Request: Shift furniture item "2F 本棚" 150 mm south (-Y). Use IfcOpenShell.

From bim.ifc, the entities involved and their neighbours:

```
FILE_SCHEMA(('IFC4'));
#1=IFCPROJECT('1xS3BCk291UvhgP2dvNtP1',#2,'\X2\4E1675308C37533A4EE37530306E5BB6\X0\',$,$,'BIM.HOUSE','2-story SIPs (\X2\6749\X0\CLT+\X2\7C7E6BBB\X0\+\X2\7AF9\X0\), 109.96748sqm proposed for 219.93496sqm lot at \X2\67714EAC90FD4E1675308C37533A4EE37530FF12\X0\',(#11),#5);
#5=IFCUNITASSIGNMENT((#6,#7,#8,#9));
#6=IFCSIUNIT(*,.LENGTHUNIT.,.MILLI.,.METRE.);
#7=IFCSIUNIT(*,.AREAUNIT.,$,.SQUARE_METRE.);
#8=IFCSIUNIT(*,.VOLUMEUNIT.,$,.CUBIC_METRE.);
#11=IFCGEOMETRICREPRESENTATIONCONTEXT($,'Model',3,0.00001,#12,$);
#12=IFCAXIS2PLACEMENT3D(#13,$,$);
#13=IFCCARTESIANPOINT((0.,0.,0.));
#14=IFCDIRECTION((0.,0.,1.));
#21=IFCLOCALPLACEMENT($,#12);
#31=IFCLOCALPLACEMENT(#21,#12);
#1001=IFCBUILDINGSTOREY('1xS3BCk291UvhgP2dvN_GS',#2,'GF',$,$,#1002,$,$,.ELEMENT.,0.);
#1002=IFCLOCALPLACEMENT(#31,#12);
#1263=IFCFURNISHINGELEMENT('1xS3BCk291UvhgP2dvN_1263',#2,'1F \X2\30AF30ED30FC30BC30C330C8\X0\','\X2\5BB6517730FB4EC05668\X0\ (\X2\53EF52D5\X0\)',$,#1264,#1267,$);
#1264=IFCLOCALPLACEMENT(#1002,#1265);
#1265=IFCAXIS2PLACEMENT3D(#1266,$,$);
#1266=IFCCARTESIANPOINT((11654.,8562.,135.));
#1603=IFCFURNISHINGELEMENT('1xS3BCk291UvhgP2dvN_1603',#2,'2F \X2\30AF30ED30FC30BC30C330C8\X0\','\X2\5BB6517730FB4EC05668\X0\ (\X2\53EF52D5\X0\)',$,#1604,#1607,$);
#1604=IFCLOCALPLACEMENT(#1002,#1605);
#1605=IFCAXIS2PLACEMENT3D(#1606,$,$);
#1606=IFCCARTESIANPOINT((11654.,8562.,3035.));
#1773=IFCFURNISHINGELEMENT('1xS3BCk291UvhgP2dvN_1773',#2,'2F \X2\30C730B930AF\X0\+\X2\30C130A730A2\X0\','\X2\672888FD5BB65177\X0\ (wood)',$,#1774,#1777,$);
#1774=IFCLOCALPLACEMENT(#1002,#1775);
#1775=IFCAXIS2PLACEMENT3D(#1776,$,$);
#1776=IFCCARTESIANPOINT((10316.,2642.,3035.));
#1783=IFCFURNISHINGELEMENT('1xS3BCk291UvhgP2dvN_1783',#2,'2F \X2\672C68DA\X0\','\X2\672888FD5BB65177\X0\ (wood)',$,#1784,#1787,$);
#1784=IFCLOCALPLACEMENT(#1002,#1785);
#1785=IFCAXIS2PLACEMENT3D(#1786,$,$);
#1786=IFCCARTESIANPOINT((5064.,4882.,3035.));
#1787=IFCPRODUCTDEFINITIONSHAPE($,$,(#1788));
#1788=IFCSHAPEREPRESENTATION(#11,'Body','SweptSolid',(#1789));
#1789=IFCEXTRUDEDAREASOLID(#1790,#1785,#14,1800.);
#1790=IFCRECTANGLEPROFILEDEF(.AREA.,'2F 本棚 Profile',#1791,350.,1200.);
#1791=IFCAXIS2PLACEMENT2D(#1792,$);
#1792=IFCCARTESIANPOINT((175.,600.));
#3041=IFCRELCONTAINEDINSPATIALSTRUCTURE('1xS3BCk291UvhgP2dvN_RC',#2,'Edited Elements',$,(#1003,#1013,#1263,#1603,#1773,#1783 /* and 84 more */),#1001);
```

```python
import ifcopenshell
import ifcopenshell.api.geometry
import ifcopenshell.util.placement
import ifcopenshell.util.unit

model = ifcopenshell.open("bim.ifc")
unit_scale = ifcopenshell.util.unit.calculate_unit_scale(model)

item = model.by_id(1783)
matrix = ifcopenshell.util.placement.get_local_placement(item.ObjectPlacement)
matrix[1, 3] -= 0.15 / unit_scale
ifcopenshell.api.geometry.edit_object_placement(model, product=item, matrix=matrix, is_si=False)

print(ifcopenshell.util.placement.get_local_placement(item.ObjectPlacement).round(3) + 0.0)

model.write("bim_updated.ifc")
```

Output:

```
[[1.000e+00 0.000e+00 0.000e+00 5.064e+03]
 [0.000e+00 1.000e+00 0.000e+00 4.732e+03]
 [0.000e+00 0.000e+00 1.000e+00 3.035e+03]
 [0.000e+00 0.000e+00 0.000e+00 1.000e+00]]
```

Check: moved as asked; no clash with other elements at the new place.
